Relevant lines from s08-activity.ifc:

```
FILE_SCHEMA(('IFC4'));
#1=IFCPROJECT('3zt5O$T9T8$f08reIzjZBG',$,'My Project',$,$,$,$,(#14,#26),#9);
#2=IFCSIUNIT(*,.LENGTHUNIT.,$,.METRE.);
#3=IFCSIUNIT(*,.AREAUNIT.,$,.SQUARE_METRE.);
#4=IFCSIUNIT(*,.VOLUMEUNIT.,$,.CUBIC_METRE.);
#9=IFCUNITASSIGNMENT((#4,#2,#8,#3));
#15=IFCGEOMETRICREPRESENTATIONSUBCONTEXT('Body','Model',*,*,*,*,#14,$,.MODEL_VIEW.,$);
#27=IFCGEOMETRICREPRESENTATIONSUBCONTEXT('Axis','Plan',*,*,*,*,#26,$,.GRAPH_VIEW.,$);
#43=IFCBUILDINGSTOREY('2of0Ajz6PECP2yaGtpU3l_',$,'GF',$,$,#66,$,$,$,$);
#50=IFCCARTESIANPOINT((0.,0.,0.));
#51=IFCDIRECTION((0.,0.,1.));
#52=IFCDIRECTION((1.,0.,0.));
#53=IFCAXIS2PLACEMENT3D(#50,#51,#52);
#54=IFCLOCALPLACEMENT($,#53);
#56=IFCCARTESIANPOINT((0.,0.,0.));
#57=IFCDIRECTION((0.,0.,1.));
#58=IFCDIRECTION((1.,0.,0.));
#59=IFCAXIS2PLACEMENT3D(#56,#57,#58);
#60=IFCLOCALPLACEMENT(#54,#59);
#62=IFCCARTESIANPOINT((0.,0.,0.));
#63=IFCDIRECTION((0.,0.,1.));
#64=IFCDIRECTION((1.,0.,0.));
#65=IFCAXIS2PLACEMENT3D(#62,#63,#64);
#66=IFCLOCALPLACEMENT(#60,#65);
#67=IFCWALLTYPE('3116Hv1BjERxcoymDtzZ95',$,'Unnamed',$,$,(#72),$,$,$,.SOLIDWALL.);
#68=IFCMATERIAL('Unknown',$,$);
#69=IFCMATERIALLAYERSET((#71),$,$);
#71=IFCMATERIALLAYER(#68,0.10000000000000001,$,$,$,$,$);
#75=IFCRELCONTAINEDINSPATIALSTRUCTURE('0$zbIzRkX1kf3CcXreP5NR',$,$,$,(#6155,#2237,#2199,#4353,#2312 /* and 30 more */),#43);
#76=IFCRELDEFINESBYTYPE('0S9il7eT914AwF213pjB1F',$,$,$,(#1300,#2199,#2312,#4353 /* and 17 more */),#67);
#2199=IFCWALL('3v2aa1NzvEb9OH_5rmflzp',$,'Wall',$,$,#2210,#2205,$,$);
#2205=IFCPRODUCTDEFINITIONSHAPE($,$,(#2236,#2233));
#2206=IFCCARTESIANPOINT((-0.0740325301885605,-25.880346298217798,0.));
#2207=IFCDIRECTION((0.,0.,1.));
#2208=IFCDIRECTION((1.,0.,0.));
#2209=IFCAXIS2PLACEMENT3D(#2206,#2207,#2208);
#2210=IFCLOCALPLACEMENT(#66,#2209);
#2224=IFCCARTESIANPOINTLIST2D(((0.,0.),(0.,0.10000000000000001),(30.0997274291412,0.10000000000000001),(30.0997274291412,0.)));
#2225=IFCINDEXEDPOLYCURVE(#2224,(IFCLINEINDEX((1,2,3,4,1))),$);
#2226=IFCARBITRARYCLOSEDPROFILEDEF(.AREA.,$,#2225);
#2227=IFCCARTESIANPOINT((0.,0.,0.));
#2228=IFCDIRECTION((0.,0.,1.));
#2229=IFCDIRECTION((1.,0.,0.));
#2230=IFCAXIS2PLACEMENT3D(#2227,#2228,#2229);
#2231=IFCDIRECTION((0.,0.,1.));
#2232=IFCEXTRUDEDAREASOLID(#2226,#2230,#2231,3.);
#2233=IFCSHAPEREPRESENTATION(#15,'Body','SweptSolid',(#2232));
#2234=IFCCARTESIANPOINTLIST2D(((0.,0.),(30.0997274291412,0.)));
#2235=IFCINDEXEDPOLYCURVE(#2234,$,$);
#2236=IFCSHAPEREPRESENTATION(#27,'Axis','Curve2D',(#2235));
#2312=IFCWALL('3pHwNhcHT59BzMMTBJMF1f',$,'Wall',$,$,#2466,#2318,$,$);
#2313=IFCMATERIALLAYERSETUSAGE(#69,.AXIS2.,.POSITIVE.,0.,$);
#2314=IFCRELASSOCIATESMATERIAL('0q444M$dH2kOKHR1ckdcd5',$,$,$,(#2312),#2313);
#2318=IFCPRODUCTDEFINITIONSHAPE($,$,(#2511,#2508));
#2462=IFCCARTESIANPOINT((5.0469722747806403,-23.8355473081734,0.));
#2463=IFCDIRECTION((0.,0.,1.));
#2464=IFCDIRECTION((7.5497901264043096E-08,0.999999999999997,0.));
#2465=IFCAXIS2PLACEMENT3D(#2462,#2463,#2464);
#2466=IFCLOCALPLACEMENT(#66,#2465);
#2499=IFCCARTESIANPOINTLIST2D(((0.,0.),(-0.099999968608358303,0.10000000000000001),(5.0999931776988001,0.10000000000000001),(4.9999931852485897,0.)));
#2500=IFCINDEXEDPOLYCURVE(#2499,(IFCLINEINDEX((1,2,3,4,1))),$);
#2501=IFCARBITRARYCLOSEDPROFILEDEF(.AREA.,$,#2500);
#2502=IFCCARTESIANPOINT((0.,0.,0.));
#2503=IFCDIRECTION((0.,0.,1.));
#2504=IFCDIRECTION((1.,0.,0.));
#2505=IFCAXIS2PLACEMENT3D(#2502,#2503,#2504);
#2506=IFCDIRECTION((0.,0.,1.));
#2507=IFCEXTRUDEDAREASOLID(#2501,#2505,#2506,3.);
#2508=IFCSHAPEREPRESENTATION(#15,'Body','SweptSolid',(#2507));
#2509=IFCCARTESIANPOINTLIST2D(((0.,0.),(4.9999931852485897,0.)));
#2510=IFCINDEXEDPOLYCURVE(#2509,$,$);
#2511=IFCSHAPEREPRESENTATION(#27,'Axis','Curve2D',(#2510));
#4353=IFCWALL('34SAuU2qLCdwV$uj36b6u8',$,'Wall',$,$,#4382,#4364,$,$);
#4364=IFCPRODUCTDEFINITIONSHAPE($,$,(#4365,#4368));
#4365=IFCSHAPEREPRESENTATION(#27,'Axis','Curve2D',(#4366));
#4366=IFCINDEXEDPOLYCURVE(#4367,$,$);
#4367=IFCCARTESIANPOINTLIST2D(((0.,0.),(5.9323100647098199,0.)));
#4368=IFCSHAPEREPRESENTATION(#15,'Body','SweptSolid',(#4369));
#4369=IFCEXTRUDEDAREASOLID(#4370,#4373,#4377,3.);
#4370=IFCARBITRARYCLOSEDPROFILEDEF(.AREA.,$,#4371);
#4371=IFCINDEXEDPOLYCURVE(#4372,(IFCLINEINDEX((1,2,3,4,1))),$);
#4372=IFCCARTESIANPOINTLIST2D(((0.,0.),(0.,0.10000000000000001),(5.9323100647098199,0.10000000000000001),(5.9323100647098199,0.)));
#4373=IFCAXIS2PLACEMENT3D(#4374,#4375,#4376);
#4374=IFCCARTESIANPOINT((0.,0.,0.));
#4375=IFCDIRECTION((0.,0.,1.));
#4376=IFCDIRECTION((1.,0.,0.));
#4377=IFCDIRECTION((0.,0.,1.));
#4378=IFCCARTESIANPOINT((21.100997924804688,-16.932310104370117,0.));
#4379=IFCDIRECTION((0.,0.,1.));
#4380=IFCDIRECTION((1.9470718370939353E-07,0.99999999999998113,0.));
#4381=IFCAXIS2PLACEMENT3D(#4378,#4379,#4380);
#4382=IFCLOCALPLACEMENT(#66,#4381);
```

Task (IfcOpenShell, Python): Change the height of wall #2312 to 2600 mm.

```python
import ifcopenshell
import ifcopenshell.geom
import ifcopenshell.util.representation
import ifcopenshell.util.shape
import ifcopenshell.util.unit

model = ifcopenshell.open("s08-activity.ifc")
unit_scale = ifcopenshell.util.unit.calculate_unit_scale(model)
settings = ifcopenshell.geom.settings()


def volume(element):
    """Net volume in cubic metres, openings subtracted."""
    shape = ifcopenshell.geom.create_shape(settings, element)
    return ifcopenshell.util.shape.get_volume(shape.geometry)


wall = model.by_guid("3pHwNhcHT59BzMMTBJMF1f")
before = volume(wall)

body = ifcopenshell.util.representation.get_representation(wall, "Model", "Body")
solid = body.Items[0]
old_height = solid.Depth
solid.Depth = 2.6 / unit_scale
after = volume(wall)

print(f"height {old_height:g} -> {solid.Depth:g}, volume {before:.3f} -> {after:.3f} m3")

model.write("s08-activity-out.ifc")
```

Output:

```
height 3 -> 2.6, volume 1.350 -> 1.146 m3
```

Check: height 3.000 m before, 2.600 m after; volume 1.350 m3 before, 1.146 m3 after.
